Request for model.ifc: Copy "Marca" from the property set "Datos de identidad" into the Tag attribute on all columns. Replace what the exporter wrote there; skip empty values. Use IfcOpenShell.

First a look at what the model holds.

```python
import ifcopenshell
import ifcopenshell.util.element

model = ifcopenshell.open("model.ifc")
print(model.schema)
columns = model.by_type("IfcColumn")
print(len(columns), "columns")
for e in columns[:8]:
    source = ifcopenshell.util.element.get_pset(e, "Datos de identidad", "Marca")
    target = e.Tag
    print(e.id(), repr(source), repr(target), sep=" | ")
```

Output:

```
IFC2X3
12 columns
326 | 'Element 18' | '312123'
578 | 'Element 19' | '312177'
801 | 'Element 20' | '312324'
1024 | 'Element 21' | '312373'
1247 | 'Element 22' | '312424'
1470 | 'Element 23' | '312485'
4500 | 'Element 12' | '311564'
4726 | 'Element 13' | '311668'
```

```python
import ifcopenshell
import ifcopenshell.util.element

model = ifcopenshell.open("model.ifc")

count = 0
for e in model.by_type("IfcColumn"):
    value = ifcopenshell.util.element.get_pset(e, "Datos de identidad", "Marca")
    current = e.Tag
    if not value or not value.strip() or current == value:
        continue
    e.Tag = value
    count += 1

print(count, "columns updated")

model.write("model_updated.ifc")
```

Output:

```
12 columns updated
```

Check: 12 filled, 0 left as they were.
